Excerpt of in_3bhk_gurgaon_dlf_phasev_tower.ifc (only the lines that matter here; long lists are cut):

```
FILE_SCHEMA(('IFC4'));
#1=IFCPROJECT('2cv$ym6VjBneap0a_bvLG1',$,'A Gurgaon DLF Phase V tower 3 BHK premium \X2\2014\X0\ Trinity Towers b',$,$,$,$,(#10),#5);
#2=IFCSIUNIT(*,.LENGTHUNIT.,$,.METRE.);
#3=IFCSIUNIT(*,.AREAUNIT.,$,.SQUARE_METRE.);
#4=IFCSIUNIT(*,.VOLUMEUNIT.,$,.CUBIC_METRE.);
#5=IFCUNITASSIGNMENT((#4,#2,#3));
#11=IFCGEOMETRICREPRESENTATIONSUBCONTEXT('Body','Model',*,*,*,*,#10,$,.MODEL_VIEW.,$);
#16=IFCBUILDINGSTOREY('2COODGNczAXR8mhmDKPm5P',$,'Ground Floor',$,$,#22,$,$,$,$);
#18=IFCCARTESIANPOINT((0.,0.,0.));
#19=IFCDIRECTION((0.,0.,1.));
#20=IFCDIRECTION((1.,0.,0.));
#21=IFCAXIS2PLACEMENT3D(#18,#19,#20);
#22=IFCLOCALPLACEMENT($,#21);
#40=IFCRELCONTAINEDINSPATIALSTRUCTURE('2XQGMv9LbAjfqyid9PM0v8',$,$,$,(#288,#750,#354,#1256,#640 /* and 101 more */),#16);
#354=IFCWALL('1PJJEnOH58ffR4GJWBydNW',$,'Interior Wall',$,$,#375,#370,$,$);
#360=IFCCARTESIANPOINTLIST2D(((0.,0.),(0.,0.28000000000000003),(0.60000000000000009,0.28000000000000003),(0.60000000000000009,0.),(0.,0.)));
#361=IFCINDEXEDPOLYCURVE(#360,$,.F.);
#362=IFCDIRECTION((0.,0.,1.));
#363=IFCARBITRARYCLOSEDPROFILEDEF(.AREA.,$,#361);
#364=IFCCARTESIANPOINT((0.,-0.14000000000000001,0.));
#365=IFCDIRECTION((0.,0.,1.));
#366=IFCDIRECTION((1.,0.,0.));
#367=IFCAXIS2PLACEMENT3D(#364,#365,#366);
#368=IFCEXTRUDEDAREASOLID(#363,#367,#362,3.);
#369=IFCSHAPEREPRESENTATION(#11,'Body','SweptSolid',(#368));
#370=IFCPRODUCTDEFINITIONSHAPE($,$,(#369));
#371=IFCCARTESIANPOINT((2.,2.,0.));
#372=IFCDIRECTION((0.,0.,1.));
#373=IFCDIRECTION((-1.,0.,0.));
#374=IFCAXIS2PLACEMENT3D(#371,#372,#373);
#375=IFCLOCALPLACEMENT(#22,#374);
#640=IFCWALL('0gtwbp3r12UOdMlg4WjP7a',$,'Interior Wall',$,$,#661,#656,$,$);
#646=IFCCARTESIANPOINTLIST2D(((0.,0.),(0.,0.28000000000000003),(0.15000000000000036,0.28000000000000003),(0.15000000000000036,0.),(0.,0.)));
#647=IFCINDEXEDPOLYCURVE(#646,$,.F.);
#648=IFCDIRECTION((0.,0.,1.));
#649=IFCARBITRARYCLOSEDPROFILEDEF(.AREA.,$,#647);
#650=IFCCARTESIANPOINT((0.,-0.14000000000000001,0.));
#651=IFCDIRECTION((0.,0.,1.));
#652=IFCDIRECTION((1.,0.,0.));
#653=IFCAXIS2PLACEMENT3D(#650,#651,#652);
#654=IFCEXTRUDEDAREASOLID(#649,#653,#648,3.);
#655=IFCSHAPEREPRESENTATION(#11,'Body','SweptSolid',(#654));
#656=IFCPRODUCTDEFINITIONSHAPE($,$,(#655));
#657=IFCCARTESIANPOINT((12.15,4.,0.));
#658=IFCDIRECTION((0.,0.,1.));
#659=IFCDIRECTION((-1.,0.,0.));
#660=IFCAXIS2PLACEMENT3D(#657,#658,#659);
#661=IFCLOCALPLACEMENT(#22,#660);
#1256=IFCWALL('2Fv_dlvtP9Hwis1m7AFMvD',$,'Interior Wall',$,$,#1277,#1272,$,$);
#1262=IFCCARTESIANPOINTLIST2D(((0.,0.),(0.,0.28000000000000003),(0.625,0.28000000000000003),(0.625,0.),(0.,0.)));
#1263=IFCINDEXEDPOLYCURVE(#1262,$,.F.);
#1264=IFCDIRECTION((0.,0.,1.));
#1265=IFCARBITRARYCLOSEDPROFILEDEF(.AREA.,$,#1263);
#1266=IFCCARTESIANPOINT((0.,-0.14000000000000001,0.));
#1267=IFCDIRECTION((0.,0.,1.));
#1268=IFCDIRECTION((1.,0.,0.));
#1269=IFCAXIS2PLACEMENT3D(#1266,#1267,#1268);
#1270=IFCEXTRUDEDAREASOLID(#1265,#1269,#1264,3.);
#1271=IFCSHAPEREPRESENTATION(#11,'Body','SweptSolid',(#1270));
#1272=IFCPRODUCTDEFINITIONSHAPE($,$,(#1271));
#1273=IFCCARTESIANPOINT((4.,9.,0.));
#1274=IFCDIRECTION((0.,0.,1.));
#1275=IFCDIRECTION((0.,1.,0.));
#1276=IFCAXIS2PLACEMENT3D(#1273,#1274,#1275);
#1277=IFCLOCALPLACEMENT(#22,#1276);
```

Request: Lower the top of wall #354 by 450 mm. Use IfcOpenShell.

```python
import ifcopenshell
import ifcopenshell.geom
import ifcopenshell.util.representation
import ifcopenshell.util.shape

model = ifcopenshell.open("in_3bhk_gurgaon_dlf_phasev_tower.ifc")
settings = ifcopenshell.geom.settings()


def volume(element):
    """Net volume in cubic metres, openings subtracted."""
    shape = ifcopenshell.geom.create_shape(settings, element)
    return ifcopenshell.util.shape.get_volume(shape.geometry)


wall = model.by_id(354)
before = volume(wall)

body = ifcopenshell.util.representation.get_representation(wall, "Model", "Body")
solid = body.Items[0]
old_height = solid.Depth
solid.Depth -= 0.45
after = volume(wall)

print(f"height {old_height:g} -> {solid.Depth:g}, volume {before:.3f} -> {after:.3f} m3")

model.write("in_3bhk_gurgaon_dlf_phasev_tower_rev.ifc")
```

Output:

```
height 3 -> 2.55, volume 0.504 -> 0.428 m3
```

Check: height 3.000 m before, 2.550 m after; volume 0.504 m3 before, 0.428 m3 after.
